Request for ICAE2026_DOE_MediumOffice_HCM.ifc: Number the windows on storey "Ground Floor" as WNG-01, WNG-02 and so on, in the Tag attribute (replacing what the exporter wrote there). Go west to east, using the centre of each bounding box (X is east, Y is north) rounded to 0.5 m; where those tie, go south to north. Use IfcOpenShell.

First a look at what the model holds.

```python
import ifcopenshell
import ifcopenshell.util.element
import ifcopenshell.util.placement

model = ifcopenshell.open("ICAE2026_DOE_MediumOffice_HCM.ifc")
print(model.schema)
storey = next(s for s in model.by_type("IfcBuildingStorey") if s.Name == "Ground Floor")
windows = [e for e in ifcopenshell.util.element.get_decomposition(storey) if e.is_a("IfcWindow")]
for e in sorted(windows, key=lambda e: e.id()):
    origin = ifcopenshell.util.placement.get_local_placement(e.ObjectPlacement)[:3, 3]
    print(e.id(), e.Tag, e.Name, origin.round(2) + 0.0, sep=" | ")
```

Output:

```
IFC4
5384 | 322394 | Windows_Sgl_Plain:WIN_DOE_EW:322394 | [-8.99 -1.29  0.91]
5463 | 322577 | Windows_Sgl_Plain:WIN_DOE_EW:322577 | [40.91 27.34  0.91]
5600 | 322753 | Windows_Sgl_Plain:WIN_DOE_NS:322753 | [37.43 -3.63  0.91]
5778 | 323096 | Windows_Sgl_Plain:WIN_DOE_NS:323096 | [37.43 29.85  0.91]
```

```python
import ifcopenshell
import ifcopenshell.geom
import ifcopenshell.util.element
import ifcopenshell.util.shape

model = ifcopenshell.open("ICAE2026_DOE_MediumOffice_HCM.ifc")
settings = ifcopenshell.geom.settings()
settings.set("use-world-coords", True)


def centre(element):
    shape = ifcopenshell.geom.create_shape(settings, element)
    return ifcopenshell.util.shape.get_bbox_centroid(shape.geometry)


storey = next(s for s in model.by_type("IfcBuildingStorey") if s.Name == "Ground Floor")
windows = [e for e in ifcopenshell.util.element.get_decomposition(storey) if e.is_a("IfcWindow")]

# Insertion points can sit at a corner or the storey origin, so sort by the geometry (in metres).
centres = {e: centre(e) for e in windows}
windows.sort(key=lambda e: (round(centres[e][0] / 0.5), centres[e][1]))

for i, e in enumerate(windows, start=1):
    number = f"WNG-{i:02d}"
    e.Tag = number
    print(e.id(), number)

model.write("ICAE2026_DOE_MediumOffice_HCM-out.ifc")
```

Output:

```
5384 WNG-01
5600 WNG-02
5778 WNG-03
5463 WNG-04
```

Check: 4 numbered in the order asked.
